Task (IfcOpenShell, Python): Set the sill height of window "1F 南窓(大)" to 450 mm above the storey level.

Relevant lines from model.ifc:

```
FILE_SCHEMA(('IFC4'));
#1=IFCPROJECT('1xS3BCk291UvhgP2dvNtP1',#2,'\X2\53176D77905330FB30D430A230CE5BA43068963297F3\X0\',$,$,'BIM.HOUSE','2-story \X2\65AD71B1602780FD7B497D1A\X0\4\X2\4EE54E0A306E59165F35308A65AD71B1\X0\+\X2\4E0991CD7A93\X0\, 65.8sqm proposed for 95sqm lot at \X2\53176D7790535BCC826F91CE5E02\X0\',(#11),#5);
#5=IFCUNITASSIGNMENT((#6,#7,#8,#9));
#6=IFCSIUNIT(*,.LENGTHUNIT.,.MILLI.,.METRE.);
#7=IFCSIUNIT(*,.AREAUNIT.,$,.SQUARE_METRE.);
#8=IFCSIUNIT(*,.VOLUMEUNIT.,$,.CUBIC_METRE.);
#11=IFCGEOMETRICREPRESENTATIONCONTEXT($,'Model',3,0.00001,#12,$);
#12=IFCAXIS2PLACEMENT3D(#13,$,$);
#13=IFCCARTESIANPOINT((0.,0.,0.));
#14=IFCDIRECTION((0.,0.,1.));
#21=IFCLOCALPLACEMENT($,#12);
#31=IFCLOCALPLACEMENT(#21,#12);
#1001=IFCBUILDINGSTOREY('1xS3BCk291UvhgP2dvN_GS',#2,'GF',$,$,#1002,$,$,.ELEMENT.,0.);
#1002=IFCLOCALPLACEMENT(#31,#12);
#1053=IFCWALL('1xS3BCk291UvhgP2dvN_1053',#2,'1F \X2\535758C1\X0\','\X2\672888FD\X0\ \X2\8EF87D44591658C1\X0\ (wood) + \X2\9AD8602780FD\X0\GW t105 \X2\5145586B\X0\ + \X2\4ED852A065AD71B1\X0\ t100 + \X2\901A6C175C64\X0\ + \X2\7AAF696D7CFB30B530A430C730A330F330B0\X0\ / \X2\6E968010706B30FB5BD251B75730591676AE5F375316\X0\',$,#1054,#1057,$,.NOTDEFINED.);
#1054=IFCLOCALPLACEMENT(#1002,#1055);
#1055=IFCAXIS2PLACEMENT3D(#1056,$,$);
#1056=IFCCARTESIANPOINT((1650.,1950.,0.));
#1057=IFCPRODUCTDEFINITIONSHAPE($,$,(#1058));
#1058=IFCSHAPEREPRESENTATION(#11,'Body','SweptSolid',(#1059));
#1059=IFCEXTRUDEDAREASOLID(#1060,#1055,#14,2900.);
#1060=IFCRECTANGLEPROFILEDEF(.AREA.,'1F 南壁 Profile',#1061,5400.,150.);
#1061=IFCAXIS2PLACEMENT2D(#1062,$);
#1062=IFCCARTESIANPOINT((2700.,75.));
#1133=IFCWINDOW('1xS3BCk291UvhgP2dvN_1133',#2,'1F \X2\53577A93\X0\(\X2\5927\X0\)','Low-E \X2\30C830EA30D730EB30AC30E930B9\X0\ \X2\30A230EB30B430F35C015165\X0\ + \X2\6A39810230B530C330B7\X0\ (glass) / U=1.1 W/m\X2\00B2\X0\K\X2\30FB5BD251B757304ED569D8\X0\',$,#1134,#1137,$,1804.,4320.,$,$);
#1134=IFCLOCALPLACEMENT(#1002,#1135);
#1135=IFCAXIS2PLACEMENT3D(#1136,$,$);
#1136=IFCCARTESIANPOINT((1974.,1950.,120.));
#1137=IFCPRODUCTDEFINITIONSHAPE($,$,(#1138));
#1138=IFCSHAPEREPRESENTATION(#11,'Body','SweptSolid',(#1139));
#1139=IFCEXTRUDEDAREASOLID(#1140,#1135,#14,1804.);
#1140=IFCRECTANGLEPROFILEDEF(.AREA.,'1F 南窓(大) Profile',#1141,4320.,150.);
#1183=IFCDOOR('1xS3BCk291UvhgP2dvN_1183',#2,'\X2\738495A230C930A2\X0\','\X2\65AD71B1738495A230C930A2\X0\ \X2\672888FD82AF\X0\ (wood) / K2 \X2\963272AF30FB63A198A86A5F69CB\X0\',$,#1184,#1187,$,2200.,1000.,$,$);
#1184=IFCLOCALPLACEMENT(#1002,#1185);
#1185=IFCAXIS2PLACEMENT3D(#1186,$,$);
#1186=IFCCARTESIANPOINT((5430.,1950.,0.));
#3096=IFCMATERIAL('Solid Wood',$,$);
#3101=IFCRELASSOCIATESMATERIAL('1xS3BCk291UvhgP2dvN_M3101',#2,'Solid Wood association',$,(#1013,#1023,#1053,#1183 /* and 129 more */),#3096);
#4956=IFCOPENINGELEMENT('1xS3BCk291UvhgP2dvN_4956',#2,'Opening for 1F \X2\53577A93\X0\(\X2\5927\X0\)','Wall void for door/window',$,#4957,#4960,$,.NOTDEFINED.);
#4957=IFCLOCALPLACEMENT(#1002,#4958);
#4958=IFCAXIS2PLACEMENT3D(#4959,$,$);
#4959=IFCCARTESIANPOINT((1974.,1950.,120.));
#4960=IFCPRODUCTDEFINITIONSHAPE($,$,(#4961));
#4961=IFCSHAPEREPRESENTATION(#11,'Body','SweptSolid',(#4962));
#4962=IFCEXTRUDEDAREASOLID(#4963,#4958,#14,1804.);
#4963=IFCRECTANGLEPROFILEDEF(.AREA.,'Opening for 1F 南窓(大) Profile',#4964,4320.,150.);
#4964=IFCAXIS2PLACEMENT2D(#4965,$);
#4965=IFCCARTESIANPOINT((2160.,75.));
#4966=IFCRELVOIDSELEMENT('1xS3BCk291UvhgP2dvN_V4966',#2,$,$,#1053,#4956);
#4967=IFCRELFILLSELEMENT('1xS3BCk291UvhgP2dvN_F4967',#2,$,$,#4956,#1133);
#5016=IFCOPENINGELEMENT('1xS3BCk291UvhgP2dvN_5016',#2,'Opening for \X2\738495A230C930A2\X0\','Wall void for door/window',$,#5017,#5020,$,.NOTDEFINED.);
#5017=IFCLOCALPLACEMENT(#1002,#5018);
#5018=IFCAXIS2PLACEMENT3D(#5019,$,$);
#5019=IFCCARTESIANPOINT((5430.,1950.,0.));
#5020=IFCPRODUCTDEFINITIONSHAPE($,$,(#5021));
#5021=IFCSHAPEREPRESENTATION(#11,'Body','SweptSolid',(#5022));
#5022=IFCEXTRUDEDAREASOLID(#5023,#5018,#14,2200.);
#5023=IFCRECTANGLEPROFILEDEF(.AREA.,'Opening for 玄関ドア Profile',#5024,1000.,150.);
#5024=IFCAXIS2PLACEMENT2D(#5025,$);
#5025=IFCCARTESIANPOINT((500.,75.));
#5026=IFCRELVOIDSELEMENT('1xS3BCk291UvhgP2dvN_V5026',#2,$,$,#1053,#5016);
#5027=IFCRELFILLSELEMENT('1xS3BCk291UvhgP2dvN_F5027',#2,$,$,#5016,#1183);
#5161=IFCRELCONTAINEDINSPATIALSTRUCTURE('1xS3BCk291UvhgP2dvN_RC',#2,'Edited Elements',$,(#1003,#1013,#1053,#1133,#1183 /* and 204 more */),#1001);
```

```python
import numpy as np
import ifcopenshell
import ifcopenshell.api.geometry
import ifcopenshell.geom
import ifcopenshell.util.element
import ifcopenshell.util.placement
import ifcopenshell.util.shape
import ifcopenshell.util.unit

model = ifcopenshell.open("model.ifc")
unit_scale = ifcopenshell.util.unit.calculate_unit_scale(model)

window = model.by_guid("1xS3BCk291UvhgP2dvN_1133")
opening = window.FillsVoids[0].RelatingOpeningElement
storey = ifcopenshell.util.element.get_container(window, ifc_class="IfcBuildingStorey")
level = ifcopenshell.util.placement.get_local_placement(storey.ObjectPlacement)[2, 3]

# The opening's origin need not be at the sill, so measure its lowest point.
shape = ifcopenshell.geom.create_shape(ifcopenshell.geom.settings(), opening)
bottom = ifcopenshell.util.shape.get_shape_bottom_elevation(shape, shape.geometry) / unit_scale
dz = level + 450.0 - bottom

shift = np.array([0.0, 0.0, dz])
# The window is not placed relative to its opening, so move both.
for product in (opening, window):
    matrix = ifcopenshell.util.placement.get_local_placement(product.ObjectPlacement)
    matrix[:3, 3] += shift
    ifcopenshell.api.geometry.edit_object_placement(model, product=product, matrix=matrix, is_si=False)

print(f"moved by {dz * unit_scale:+.3f} m")

model.write("model_rev.ifc")
```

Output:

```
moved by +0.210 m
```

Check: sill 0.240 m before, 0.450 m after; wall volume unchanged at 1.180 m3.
